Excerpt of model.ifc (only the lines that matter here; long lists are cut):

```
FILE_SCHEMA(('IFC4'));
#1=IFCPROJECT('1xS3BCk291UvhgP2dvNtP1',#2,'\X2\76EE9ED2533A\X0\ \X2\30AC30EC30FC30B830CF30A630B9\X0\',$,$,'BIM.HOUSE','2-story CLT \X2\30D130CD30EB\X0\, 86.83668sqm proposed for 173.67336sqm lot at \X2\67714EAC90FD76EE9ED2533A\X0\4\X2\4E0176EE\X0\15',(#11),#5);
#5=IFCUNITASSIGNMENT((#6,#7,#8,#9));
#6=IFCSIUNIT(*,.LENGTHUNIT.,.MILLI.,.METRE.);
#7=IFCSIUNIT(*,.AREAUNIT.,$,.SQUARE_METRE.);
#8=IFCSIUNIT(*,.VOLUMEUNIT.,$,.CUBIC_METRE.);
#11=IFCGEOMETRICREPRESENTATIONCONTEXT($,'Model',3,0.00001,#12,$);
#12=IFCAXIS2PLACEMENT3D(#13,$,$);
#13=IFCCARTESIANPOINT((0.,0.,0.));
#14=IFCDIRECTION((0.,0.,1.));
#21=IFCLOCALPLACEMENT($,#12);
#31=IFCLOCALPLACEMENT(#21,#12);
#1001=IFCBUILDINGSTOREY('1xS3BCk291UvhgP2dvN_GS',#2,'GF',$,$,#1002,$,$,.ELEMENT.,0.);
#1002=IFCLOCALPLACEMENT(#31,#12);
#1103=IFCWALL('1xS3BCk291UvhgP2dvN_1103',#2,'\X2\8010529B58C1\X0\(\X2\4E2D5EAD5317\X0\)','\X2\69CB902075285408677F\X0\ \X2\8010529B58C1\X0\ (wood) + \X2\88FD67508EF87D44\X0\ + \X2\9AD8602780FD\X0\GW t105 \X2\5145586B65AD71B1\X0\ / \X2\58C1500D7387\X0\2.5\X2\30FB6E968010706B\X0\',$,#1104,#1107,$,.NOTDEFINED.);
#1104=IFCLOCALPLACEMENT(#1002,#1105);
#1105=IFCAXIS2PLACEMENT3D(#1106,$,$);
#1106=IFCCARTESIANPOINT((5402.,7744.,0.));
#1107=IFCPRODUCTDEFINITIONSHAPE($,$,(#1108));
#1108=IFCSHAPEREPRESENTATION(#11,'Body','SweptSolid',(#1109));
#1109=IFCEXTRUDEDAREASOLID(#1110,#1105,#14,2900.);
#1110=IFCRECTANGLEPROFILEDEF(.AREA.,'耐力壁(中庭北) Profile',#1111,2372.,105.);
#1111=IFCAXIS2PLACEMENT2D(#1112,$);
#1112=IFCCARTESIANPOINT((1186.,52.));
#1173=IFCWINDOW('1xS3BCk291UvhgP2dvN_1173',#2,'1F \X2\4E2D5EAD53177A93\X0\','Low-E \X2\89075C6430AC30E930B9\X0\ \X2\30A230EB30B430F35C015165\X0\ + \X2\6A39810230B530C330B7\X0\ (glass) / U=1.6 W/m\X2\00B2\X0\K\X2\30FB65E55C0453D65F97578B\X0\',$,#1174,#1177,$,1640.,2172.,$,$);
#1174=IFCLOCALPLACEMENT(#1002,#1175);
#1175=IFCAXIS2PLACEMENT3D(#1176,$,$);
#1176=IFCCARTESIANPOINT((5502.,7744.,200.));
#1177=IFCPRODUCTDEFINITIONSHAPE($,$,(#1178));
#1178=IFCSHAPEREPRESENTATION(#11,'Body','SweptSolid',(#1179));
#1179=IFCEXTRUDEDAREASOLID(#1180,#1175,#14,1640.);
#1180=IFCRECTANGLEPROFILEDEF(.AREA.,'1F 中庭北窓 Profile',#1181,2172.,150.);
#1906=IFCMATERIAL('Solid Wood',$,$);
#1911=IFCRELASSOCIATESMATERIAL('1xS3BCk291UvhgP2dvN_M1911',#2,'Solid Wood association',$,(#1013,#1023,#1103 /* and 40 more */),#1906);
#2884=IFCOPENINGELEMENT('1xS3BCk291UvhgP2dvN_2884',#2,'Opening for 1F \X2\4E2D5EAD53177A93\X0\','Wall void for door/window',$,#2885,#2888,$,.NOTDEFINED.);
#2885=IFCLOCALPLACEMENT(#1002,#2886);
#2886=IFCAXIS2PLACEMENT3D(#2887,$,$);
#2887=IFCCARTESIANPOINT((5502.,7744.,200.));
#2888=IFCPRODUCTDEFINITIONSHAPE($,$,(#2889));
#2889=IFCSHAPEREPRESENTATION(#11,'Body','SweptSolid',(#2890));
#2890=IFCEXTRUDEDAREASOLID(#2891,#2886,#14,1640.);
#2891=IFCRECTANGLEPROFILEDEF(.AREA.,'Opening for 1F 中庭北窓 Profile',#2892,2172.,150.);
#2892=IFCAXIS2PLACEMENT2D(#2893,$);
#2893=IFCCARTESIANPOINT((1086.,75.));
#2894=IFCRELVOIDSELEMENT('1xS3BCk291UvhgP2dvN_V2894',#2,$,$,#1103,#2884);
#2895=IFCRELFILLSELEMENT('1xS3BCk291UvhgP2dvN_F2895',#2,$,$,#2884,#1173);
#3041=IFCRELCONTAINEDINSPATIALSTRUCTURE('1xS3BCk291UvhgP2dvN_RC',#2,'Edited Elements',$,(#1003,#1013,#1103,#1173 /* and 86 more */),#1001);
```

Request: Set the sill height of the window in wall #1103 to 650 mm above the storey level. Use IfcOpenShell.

```python
import numpy as np
import ifcopenshell
import ifcopenshell.api.geometry
import ifcopenshell.geom
import ifcopenshell.util.element
import ifcopenshell.util.placement
import ifcopenshell.util.shape
import ifcopenshell.util.unit

model = ifcopenshell.open("model.ifc")
unit_scale = ifcopenshell.util.unit.calculate_unit_scale(model)

window = model.by_id(1173)
opening = window.FillsVoids[0].RelatingOpeningElement
storey = ifcopenshell.util.element.get_container(window, ifc_class="IfcBuildingStorey")
level = ifcopenshell.util.placement.get_local_placement(storey.ObjectPlacement)[2, 3]

# The opening's origin need not be at the sill, so measure its lowest point.
shape = ifcopenshell.geom.create_shape(ifcopenshell.geom.settings(), opening)
bottom = ifcopenshell.util.shape.get_shape_bottom_elevation(shape, shape.geometry) / unit_scale
dz = level + 650.0 - bottom

shift = np.array([0.0, 0.0, dz])
# The window is not placed relative to its opening, so move both.
for product in (opening, window):
    matrix = ifcopenshell.util.placement.get_local_placement(product.ObjectPlacement)
    matrix[:3, 3] += shift
    ifcopenshell.api.geometry.edit_object_placement(model, product=product, matrix=matrix, is_si=False)

print(f"moved by {dz * unit_scale:+.3f} m")

model.write("model_v2.ifc")
```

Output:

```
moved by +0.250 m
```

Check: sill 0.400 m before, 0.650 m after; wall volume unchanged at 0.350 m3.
